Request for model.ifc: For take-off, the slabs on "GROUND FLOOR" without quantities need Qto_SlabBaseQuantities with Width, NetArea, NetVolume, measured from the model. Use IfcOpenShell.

First a look at what the model holds.

```python
import ifcopenshell
import ifcopenshell.util.element
import ifcopenshell.util.unit

model = ifcopenshell.open("model.ifc")
print(model.schema)
for unit_type in ("LENGTHUNIT", "AREAUNIT", "VOLUMEUNIT"):
    print(unit_type, ifcopenshell.util.unit.calculate_unit_scale(model, unit_type))
storey = next(s for s in model.by_type("IfcBuildingStorey") if s.Name == "GROUND FLOOR")
slabs = [e for e in ifcopenshell.util.element.get_decomposition(storey) if e.is_a("IfcSlab")]
for e in sorted(slabs, key=lambda e: e.id()):
    print(e.id(), e.is_a(), e.Name, list(ifcopenshell.util.element.get_psets(e, qtos_only=True)), sep=" | ")
```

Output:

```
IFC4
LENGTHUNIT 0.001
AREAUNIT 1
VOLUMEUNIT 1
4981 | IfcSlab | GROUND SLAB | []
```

```python
import ifcopenshell
import ifcopenshell.api.pset
import ifcopenshell.geom
import ifcopenshell.util.element
import ifcopenshell.util.shape
import ifcopenshell.util.unit

model = ifcopenshell.open("model.ifc")
unit_scale = ifcopenshell.util.unit.calculate_unit_scale(model)
area_scale = ifcopenshell.util.unit.calculate_unit_scale(model, "AREAUNIT")
volume_scale = ifcopenshell.util.unit.calculate_unit_scale(model, "VOLUMEUNIT")
settings = ifcopenshell.geom.settings()

storey = next(s for s in model.by_type("IfcBuildingStorey") if s.Name == "GROUND FLOOR")
slabs = [e for e in ifcopenshell.util.element.get_decomposition(storey) if e.is_a("IfcSlab")]

for e in sorted(slabs, key=lambda e: e.id()):
    if ifcopenshell.util.element.get_psets(e, qtos_only=True, should_inherit=False):
        continue
    # Geometry comes back in metres, in the element's own axes.
    shape = ifcopenshell.geom.create_shape(settings, e)
    values = {
        "Width": ifcopenshell.util.shape.get_z(shape.geometry) / unit_scale,
        "NetArea": ifcopenshell.util.shape.get_footprint_area(shape.geometry) / area_scale,
        "NetVolume": ifcopenshell.util.shape.get_volume(shape.geometry) / volume_scale,
    }
    qto = ifcopenshell.api.pset.add_qto(model, product=e, name="Qto_SlabBaseQuantities")
    ifcopenshell.api.pset.edit_qto(model, qto=qto, properties=values)
    print(e.id(), {k: round(v, 3) for k, v in values.items()})

model.write("model_rev.ifc")
```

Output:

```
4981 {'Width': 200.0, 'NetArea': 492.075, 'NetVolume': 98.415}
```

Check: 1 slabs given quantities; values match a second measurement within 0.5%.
